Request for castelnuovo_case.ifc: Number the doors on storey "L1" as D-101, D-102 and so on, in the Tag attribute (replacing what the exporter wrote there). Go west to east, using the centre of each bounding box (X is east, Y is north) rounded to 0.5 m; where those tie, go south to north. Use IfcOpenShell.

First a look at what the model holds.

```python
import ifcopenshell
import ifcopenshell.util.element
import ifcopenshell.util.placement

model = ifcopenshell.open("castelnuovo_case.ifc")
print(model.schema)
storey = next(s for s in model.by_type("IfcBuildingStorey") if s.Name == "L1")
doors = [e for e in ifcopenshell.util.element.get_decomposition(storey) if e.is_a("IfcDoor")]
for e in sorted(doors, key=lambda e: e.id()):
    origin = ifcopenshell.util.placement.get_local_placement(e.ObjectPlacement)[:3, 3]
    print(e.id(), e.Tag, e.Name, origin.round(2) + 0.0, sep=" | ")
```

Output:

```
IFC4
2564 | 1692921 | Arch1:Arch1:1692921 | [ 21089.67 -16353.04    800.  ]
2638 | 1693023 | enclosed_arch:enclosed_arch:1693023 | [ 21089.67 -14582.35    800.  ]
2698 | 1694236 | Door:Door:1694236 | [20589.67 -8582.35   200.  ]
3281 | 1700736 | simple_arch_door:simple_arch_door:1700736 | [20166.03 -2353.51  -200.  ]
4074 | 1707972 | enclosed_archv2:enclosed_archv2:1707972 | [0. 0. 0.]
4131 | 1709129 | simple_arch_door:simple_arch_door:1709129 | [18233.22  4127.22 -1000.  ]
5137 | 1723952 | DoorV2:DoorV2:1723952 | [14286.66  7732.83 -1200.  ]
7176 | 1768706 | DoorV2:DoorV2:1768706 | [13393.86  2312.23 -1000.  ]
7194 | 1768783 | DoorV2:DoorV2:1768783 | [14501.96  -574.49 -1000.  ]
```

```python
import ifcopenshell
import ifcopenshell.geom
import ifcopenshell.util.element
import ifcopenshell.util.shape

model = ifcopenshell.open("castelnuovo_case.ifc")
settings = ifcopenshell.geom.settings()
settings.set("use-world-coords", True)


def centre(element):
    shape = ifcopenshell.geom.create_shape(settings, element)
    return ifcopenshell.util.shape.get_bbox_centroid(shape.geometry)


storey = next(s for s in model.by_type("IfcBuildingStorey") if s.Name == "L1")
doors = [e for e in ifcopenshell.util.element.get_decomposition(storey) if e.is_a("IfcDoor")]

# Insertion points can sit at a corner or the storey origin, so sort by the geometry (in metres).
centres = {e: centre(e) for e in doors}
doors.sort(key=lambda e: (round(centres[e][0] / 0.5), centres[e][1]))

for i, e in enumerate(doors, start=1):
    number = f"D-1{i:02d}"
    e.Tag = number
    print(e.id(), number)

model.write("castelnuovo_case_rev.ifc")
```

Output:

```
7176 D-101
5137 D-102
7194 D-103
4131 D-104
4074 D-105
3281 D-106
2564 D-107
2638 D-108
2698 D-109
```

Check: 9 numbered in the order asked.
